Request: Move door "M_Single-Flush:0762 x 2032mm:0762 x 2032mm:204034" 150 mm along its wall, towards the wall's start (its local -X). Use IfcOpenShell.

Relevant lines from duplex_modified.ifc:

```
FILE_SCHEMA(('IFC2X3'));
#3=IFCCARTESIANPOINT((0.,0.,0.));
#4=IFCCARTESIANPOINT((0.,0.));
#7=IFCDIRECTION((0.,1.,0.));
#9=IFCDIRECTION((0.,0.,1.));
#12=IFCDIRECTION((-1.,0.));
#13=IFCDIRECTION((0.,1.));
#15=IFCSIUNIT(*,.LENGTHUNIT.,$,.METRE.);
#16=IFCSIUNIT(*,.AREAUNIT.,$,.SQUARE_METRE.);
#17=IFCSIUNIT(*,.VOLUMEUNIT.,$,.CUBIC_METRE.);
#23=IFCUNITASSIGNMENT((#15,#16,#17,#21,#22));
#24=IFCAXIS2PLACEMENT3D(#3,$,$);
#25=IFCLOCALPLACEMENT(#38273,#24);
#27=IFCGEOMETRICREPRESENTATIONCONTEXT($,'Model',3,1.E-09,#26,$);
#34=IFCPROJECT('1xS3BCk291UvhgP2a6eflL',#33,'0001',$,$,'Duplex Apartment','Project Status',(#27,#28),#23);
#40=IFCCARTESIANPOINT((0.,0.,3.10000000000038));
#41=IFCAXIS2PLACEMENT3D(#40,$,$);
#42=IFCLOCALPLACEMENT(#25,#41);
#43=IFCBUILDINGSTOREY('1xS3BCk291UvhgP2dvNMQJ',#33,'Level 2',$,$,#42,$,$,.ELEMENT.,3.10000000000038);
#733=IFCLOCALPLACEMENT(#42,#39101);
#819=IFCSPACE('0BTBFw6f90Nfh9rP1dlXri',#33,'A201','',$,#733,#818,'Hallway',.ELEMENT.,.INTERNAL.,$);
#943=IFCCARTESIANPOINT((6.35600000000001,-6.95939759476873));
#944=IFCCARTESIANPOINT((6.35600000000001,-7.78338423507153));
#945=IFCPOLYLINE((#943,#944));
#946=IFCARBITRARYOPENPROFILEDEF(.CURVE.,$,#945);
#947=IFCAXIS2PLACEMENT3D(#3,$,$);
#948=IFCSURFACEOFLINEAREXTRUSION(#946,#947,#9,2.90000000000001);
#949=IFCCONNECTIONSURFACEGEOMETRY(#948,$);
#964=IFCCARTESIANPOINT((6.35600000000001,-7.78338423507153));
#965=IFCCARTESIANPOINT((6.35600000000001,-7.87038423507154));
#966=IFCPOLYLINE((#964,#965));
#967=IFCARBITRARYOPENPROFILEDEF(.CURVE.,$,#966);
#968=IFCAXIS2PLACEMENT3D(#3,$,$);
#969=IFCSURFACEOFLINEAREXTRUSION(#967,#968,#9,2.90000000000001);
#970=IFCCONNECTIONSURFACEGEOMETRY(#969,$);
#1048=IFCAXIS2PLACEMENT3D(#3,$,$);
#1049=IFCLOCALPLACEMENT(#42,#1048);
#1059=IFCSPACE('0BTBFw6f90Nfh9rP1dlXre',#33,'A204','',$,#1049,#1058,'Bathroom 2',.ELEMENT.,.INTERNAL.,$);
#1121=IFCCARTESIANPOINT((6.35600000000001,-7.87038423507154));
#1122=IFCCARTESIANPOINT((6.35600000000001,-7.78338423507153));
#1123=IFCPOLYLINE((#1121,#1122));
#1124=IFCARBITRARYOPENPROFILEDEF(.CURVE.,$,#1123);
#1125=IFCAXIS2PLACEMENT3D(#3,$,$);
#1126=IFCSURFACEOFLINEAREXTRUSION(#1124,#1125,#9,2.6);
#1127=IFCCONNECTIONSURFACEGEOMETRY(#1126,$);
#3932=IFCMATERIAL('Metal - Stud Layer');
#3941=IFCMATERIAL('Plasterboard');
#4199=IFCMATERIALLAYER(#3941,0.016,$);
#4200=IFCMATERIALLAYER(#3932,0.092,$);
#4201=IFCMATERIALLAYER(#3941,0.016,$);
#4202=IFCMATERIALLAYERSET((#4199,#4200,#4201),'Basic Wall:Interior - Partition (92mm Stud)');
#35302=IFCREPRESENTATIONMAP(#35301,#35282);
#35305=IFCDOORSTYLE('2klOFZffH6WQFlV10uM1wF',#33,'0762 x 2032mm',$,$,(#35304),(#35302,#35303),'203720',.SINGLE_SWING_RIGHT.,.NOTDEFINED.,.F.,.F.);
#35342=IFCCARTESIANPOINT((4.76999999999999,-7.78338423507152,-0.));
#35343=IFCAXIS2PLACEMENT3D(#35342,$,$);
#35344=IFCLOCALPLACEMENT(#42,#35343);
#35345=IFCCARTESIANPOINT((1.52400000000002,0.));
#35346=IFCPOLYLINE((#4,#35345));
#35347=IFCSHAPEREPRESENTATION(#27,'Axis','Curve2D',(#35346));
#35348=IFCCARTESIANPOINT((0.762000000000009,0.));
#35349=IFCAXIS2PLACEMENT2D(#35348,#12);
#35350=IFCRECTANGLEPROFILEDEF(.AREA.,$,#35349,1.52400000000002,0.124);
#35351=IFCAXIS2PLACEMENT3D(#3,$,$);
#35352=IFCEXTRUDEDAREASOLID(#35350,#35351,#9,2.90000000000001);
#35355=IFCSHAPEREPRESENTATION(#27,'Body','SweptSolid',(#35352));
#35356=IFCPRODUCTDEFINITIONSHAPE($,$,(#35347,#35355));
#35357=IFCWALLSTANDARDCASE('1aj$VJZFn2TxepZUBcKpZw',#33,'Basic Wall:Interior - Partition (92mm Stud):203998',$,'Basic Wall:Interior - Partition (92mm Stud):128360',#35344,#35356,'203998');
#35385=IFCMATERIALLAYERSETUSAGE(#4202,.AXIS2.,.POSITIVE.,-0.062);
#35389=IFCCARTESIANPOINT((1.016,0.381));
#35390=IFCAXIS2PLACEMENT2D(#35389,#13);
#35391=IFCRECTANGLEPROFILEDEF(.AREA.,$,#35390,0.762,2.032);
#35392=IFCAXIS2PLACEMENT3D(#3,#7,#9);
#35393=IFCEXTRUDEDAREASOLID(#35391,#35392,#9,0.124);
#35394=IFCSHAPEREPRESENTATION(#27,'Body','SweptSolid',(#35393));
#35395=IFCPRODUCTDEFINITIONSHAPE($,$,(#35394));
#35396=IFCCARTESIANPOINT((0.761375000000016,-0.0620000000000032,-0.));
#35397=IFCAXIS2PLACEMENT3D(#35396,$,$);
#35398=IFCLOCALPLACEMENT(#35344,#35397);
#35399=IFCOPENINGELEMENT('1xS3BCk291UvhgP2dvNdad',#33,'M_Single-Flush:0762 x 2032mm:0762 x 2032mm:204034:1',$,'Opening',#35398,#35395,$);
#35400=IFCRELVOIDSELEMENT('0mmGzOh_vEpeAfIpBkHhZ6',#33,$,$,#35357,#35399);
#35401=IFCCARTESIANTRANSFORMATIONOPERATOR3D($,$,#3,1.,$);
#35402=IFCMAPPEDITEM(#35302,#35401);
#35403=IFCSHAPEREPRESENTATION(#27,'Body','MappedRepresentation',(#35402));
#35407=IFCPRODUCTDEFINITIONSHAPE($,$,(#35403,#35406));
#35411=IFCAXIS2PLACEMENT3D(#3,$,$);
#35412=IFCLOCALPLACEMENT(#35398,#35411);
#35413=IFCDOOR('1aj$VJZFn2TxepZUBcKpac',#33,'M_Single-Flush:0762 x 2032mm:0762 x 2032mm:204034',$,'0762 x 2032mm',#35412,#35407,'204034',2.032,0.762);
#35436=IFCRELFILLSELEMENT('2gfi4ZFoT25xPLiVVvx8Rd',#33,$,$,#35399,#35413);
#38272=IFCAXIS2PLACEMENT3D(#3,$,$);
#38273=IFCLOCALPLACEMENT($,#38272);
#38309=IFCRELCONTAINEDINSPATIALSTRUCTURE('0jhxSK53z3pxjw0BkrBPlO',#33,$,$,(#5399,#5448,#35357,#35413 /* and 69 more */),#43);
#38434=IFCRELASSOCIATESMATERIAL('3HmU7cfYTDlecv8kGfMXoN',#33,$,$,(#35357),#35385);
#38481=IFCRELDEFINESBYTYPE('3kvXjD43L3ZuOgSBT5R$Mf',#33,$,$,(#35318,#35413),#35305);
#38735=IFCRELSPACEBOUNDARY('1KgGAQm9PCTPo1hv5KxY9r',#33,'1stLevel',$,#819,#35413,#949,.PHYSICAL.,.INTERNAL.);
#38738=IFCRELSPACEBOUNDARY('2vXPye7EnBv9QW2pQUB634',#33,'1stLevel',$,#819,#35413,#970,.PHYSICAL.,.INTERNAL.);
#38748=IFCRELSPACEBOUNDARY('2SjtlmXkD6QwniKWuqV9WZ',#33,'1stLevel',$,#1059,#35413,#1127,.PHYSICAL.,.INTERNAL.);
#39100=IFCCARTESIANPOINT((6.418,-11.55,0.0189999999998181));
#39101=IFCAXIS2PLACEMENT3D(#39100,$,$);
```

```python
import numpy as np
import ifcopenshell
import ifcopenshell.api.geometry
import ifcopenshell.util.placement

model = ifcopenshell.open("duplex_modified.ifc")

door = model.by_guid("1aj$VJZFn2TxepZUBcKpac")
opening = door.FillsVoids[0].RelatingOpeningElement
wall = opening.VoidsElements[0].RelatingBuildingElement

wall_matrix = ifcopenshell.util.placement.get_local_placement(wall.ObjectPlacement)
shift = wall_matrix[:3, 0] * -0.15
before = ifcopenshell.util.placement.get_local_placement(door.ObjectPlacement)[:3, 3].copy()

# The door is placed relative to its opening, so it follows when the opening moves.
matrix = ifcopenshell.util.placement.get_local_placement(opening.ObjectPlacement)
matrix[:3, 3] += shift
ifcopenshell.api.geometry.edit_object_placement(
    model, product=opening, matrix=matrix, is_si=False, should_transform_children=True
)

# Space boundary surfaces are stored in each space's coordinates; move them too.
for rel in door.ProvidesBoundaries:
    if not rel.ConnectionGeometry:
        continue
    surface = rel.ConnectionGeometry.SurfaceOnRelatingElement
    space_matrix = ifcopenshell.util.placement.get_local_placement(rel.RelatingSpace.ObjectPlacement)
    point = np.array(surface.Position.Location.Coordinates) + space_matrix[:3, :3].T @ shift
    surface.Position = model.createIfcAxis2Placement3D(
        model.createIfcCartesianPoint(point.tolist()), surface.Position.Axis, surface.Position.RefDirection
    )

after = ifcopenshell.util.placement.get_local_placement(door.ObjectPlacement)[:3, 3]
print("door moved by", (after - before).round(3) + 0.0)

model.write("duplex_modified_edited.ifc")
```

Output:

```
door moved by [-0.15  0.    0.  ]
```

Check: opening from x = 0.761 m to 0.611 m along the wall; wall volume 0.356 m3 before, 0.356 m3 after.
